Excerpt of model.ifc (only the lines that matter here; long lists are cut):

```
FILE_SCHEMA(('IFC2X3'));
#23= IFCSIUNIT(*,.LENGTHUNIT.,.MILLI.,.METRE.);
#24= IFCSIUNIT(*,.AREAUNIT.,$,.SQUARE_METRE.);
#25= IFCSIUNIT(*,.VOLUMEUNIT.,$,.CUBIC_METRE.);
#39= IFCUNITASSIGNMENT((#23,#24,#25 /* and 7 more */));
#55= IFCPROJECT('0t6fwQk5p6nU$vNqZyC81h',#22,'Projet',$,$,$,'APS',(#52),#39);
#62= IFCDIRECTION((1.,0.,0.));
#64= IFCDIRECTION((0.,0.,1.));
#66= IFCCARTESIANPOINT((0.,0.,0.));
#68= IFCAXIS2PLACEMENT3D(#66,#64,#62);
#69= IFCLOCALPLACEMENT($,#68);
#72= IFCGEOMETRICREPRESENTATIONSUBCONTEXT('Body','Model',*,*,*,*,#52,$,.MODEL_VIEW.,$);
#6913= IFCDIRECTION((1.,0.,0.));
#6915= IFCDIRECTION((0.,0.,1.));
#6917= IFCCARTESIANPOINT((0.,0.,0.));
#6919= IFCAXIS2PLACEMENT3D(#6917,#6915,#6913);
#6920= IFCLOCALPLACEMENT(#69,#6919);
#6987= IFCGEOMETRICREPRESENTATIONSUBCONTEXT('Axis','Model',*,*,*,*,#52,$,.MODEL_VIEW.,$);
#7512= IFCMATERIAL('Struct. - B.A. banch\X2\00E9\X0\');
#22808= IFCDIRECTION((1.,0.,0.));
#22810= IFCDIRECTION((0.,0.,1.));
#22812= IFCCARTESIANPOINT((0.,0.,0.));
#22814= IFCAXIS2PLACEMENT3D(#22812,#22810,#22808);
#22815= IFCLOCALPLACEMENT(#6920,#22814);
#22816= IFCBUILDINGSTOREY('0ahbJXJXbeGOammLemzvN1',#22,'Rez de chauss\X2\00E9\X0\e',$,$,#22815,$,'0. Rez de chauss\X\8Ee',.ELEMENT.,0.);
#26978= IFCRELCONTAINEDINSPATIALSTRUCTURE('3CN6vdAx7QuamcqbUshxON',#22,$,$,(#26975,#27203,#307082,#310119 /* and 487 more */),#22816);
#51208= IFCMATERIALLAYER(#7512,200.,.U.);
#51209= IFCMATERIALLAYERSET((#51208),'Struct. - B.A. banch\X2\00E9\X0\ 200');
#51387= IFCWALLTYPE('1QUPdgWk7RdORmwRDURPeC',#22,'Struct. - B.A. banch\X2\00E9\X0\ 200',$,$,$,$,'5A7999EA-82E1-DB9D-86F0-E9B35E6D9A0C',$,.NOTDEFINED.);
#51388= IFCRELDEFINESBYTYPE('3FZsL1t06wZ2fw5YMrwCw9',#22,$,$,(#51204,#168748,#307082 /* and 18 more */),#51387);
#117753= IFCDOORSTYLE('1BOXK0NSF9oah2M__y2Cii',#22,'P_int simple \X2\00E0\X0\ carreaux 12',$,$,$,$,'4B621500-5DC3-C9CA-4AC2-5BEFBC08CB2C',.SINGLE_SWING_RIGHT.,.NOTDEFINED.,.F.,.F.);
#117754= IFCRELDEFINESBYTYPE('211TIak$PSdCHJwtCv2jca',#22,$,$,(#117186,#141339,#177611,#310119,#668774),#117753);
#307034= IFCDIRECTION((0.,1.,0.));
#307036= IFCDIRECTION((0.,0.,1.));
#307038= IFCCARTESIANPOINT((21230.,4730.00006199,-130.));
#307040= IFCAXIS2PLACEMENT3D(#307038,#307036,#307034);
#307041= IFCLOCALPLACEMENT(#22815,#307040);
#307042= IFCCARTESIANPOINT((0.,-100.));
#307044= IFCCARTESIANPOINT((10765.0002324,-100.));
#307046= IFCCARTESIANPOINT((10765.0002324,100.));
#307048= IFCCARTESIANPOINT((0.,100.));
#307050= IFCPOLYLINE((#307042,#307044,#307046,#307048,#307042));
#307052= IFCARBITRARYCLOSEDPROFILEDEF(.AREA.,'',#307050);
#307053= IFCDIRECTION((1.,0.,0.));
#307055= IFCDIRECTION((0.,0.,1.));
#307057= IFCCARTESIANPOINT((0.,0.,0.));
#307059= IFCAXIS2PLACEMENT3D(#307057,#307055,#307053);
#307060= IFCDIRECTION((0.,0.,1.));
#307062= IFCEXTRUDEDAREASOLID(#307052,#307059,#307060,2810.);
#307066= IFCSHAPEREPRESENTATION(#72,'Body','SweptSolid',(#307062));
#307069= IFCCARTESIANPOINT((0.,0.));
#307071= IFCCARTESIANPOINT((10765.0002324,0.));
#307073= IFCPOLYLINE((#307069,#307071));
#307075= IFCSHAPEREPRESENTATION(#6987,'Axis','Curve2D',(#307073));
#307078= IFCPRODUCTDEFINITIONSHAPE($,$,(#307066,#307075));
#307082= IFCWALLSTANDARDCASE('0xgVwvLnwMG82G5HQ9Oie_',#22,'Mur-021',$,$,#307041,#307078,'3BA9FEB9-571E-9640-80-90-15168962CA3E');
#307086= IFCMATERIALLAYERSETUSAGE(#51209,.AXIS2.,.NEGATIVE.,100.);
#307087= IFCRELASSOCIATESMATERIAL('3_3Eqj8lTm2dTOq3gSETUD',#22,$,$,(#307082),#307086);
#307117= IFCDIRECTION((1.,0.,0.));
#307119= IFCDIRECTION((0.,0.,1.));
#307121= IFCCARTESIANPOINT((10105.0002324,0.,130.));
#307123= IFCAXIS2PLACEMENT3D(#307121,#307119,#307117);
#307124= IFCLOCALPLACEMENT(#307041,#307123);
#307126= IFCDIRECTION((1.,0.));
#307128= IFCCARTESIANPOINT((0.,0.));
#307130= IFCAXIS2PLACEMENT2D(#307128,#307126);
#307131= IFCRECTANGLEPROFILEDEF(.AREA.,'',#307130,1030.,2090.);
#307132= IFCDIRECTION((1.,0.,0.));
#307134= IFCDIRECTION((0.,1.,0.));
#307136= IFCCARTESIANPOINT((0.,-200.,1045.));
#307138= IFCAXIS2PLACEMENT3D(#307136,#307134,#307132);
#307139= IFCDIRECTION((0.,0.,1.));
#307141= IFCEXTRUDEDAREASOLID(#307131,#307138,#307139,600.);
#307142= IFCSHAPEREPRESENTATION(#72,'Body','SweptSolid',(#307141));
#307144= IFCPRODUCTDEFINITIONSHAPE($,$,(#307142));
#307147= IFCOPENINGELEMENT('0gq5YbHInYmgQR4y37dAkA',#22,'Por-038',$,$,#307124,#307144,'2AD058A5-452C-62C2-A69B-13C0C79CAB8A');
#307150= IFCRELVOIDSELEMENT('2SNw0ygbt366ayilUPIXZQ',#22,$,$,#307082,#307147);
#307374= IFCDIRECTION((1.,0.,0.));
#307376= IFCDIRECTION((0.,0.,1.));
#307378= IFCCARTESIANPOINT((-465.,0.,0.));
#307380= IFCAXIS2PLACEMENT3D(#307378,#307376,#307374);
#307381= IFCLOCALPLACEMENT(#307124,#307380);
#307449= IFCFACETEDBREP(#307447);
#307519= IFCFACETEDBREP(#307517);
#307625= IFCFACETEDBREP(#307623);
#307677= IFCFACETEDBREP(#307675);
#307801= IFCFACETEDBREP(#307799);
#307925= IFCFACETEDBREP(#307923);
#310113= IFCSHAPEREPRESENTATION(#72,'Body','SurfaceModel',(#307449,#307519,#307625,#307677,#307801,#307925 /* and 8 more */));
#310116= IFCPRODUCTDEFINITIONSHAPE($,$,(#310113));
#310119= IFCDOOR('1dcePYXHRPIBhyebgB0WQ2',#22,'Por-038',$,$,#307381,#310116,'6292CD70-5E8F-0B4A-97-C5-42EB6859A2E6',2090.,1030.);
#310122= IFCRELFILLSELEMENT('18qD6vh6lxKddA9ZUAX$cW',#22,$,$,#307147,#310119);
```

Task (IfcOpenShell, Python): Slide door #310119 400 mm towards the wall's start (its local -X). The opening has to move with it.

```python
import ifcopenshell
import ifcopenshell.api.geometry
import ifcopenshell.util.placement
import ifcopenshell.util.unit

model = ifcopenshell.open("model.ifc")
unit_scale = ifcopenshell.util.unit.calculate_unit_scale(model)

door = model.by_guid("1dcePYXHRPIBhyebgB0WQ2")
opening = door.FillsVoids[0].RelatingOpeningElement
wall = opening.VoidsElements[0].RelatingBuildingElement

wall_matrix = ifcopenshell.util.placement.get_local_placement(wall.ObjectPlacement)
shift = wall_matrix[:3, 0] * -0.4 / unit_scale
before = ifcopenshell.util.placement.get_local_placement(door.ObjectPlacement)[:3, 3].copy()

# The door is placed relative to its opening, so it follows when the opening moves.
matrix = ifcopenshell.util.placement.get_local_placement(opening.ObjectPlacement)
matrix[:3, 3] += shift
ifcopenshell.api.geometry.edit_object_placement(
    model, product=opening, matrix=matrix, is_si=False, should_transform_children=True
)

after = ifcopenshell.util.placement.get_local_placement(door.ObjectPlacement)[:3, 3]
print("door moved by", (after - before).round(3) + 0.0)

model.write("model_rev.ifc")
```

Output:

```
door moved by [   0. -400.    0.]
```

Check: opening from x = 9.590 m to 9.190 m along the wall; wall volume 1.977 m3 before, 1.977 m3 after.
